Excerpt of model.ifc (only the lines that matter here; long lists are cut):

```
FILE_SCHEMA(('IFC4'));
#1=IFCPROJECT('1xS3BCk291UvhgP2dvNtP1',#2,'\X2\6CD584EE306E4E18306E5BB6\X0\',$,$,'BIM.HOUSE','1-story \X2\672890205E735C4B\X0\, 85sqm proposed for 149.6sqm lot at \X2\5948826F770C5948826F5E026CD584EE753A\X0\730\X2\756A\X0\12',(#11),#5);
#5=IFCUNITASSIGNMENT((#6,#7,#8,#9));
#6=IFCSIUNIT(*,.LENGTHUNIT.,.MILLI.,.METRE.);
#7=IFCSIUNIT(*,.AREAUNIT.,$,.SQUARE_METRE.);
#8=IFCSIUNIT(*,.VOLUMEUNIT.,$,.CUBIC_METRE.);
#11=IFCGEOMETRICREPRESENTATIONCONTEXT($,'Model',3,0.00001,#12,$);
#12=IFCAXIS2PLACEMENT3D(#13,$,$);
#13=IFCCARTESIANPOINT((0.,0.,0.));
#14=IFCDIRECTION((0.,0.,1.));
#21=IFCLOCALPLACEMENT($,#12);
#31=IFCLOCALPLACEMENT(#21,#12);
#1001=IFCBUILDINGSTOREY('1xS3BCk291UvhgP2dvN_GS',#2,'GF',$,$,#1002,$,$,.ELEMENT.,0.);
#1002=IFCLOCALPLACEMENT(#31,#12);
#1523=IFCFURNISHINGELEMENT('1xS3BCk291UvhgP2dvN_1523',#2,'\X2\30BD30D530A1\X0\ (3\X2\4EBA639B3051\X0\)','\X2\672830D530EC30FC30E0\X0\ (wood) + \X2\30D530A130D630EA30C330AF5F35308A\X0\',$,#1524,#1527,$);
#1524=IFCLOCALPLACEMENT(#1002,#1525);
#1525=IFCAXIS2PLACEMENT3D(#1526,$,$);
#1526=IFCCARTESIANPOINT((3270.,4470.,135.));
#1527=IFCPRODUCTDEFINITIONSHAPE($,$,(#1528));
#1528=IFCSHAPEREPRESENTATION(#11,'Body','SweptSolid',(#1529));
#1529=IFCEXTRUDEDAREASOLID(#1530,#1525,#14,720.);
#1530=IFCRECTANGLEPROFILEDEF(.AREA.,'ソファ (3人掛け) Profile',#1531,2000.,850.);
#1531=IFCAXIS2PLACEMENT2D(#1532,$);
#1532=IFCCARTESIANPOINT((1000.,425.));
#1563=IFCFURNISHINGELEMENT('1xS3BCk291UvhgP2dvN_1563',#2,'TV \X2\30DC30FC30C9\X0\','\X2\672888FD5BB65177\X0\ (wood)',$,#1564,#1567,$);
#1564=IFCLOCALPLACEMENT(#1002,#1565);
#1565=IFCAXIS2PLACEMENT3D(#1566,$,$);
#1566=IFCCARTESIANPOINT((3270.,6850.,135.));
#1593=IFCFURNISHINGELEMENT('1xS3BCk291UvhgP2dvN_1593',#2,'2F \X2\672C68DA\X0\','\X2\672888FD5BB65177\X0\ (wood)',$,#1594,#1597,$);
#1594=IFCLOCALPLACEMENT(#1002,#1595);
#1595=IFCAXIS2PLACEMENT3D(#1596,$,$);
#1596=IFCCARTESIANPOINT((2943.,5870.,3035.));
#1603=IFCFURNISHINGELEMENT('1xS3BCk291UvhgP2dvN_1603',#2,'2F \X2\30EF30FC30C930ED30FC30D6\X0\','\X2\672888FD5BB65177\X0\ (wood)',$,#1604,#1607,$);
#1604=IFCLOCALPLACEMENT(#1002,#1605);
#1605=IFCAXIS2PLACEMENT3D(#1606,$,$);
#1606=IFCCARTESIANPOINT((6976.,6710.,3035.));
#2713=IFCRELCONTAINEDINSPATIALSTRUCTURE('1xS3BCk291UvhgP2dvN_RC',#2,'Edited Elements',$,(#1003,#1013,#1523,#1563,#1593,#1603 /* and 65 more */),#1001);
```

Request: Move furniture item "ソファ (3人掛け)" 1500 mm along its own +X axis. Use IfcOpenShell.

```python
import ifcopenshell
import ifcopenshell.api.geometry
import ifcopenshell.util.placement
import ifcopenshell.util.unit

model = ifcopenshell.open("model.ifc")
unit_scale = ifcopenshell.util.unit.calculate_unit_scale(model)

item = model.by_id(1523)
matrix = ifcopenshell.util.placement.get_local_placement(item.ObjectPlacement)
matrix[:3, 3] += matrix[:3, 0] * 1.5 / unit_scale
ifcopenshell.api.geometry.edit_object_placement(model, product=item, matrix=matrix, is_si=False)

print(ifcopenshell.util.placement.get_local_placement(item.ObjectPlacement).round(3) + 0.0)

model.write("model_updated.ifc")
```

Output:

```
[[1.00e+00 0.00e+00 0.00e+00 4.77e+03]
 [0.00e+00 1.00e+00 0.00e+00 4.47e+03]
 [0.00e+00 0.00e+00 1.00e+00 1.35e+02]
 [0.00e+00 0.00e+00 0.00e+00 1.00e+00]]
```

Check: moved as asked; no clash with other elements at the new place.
